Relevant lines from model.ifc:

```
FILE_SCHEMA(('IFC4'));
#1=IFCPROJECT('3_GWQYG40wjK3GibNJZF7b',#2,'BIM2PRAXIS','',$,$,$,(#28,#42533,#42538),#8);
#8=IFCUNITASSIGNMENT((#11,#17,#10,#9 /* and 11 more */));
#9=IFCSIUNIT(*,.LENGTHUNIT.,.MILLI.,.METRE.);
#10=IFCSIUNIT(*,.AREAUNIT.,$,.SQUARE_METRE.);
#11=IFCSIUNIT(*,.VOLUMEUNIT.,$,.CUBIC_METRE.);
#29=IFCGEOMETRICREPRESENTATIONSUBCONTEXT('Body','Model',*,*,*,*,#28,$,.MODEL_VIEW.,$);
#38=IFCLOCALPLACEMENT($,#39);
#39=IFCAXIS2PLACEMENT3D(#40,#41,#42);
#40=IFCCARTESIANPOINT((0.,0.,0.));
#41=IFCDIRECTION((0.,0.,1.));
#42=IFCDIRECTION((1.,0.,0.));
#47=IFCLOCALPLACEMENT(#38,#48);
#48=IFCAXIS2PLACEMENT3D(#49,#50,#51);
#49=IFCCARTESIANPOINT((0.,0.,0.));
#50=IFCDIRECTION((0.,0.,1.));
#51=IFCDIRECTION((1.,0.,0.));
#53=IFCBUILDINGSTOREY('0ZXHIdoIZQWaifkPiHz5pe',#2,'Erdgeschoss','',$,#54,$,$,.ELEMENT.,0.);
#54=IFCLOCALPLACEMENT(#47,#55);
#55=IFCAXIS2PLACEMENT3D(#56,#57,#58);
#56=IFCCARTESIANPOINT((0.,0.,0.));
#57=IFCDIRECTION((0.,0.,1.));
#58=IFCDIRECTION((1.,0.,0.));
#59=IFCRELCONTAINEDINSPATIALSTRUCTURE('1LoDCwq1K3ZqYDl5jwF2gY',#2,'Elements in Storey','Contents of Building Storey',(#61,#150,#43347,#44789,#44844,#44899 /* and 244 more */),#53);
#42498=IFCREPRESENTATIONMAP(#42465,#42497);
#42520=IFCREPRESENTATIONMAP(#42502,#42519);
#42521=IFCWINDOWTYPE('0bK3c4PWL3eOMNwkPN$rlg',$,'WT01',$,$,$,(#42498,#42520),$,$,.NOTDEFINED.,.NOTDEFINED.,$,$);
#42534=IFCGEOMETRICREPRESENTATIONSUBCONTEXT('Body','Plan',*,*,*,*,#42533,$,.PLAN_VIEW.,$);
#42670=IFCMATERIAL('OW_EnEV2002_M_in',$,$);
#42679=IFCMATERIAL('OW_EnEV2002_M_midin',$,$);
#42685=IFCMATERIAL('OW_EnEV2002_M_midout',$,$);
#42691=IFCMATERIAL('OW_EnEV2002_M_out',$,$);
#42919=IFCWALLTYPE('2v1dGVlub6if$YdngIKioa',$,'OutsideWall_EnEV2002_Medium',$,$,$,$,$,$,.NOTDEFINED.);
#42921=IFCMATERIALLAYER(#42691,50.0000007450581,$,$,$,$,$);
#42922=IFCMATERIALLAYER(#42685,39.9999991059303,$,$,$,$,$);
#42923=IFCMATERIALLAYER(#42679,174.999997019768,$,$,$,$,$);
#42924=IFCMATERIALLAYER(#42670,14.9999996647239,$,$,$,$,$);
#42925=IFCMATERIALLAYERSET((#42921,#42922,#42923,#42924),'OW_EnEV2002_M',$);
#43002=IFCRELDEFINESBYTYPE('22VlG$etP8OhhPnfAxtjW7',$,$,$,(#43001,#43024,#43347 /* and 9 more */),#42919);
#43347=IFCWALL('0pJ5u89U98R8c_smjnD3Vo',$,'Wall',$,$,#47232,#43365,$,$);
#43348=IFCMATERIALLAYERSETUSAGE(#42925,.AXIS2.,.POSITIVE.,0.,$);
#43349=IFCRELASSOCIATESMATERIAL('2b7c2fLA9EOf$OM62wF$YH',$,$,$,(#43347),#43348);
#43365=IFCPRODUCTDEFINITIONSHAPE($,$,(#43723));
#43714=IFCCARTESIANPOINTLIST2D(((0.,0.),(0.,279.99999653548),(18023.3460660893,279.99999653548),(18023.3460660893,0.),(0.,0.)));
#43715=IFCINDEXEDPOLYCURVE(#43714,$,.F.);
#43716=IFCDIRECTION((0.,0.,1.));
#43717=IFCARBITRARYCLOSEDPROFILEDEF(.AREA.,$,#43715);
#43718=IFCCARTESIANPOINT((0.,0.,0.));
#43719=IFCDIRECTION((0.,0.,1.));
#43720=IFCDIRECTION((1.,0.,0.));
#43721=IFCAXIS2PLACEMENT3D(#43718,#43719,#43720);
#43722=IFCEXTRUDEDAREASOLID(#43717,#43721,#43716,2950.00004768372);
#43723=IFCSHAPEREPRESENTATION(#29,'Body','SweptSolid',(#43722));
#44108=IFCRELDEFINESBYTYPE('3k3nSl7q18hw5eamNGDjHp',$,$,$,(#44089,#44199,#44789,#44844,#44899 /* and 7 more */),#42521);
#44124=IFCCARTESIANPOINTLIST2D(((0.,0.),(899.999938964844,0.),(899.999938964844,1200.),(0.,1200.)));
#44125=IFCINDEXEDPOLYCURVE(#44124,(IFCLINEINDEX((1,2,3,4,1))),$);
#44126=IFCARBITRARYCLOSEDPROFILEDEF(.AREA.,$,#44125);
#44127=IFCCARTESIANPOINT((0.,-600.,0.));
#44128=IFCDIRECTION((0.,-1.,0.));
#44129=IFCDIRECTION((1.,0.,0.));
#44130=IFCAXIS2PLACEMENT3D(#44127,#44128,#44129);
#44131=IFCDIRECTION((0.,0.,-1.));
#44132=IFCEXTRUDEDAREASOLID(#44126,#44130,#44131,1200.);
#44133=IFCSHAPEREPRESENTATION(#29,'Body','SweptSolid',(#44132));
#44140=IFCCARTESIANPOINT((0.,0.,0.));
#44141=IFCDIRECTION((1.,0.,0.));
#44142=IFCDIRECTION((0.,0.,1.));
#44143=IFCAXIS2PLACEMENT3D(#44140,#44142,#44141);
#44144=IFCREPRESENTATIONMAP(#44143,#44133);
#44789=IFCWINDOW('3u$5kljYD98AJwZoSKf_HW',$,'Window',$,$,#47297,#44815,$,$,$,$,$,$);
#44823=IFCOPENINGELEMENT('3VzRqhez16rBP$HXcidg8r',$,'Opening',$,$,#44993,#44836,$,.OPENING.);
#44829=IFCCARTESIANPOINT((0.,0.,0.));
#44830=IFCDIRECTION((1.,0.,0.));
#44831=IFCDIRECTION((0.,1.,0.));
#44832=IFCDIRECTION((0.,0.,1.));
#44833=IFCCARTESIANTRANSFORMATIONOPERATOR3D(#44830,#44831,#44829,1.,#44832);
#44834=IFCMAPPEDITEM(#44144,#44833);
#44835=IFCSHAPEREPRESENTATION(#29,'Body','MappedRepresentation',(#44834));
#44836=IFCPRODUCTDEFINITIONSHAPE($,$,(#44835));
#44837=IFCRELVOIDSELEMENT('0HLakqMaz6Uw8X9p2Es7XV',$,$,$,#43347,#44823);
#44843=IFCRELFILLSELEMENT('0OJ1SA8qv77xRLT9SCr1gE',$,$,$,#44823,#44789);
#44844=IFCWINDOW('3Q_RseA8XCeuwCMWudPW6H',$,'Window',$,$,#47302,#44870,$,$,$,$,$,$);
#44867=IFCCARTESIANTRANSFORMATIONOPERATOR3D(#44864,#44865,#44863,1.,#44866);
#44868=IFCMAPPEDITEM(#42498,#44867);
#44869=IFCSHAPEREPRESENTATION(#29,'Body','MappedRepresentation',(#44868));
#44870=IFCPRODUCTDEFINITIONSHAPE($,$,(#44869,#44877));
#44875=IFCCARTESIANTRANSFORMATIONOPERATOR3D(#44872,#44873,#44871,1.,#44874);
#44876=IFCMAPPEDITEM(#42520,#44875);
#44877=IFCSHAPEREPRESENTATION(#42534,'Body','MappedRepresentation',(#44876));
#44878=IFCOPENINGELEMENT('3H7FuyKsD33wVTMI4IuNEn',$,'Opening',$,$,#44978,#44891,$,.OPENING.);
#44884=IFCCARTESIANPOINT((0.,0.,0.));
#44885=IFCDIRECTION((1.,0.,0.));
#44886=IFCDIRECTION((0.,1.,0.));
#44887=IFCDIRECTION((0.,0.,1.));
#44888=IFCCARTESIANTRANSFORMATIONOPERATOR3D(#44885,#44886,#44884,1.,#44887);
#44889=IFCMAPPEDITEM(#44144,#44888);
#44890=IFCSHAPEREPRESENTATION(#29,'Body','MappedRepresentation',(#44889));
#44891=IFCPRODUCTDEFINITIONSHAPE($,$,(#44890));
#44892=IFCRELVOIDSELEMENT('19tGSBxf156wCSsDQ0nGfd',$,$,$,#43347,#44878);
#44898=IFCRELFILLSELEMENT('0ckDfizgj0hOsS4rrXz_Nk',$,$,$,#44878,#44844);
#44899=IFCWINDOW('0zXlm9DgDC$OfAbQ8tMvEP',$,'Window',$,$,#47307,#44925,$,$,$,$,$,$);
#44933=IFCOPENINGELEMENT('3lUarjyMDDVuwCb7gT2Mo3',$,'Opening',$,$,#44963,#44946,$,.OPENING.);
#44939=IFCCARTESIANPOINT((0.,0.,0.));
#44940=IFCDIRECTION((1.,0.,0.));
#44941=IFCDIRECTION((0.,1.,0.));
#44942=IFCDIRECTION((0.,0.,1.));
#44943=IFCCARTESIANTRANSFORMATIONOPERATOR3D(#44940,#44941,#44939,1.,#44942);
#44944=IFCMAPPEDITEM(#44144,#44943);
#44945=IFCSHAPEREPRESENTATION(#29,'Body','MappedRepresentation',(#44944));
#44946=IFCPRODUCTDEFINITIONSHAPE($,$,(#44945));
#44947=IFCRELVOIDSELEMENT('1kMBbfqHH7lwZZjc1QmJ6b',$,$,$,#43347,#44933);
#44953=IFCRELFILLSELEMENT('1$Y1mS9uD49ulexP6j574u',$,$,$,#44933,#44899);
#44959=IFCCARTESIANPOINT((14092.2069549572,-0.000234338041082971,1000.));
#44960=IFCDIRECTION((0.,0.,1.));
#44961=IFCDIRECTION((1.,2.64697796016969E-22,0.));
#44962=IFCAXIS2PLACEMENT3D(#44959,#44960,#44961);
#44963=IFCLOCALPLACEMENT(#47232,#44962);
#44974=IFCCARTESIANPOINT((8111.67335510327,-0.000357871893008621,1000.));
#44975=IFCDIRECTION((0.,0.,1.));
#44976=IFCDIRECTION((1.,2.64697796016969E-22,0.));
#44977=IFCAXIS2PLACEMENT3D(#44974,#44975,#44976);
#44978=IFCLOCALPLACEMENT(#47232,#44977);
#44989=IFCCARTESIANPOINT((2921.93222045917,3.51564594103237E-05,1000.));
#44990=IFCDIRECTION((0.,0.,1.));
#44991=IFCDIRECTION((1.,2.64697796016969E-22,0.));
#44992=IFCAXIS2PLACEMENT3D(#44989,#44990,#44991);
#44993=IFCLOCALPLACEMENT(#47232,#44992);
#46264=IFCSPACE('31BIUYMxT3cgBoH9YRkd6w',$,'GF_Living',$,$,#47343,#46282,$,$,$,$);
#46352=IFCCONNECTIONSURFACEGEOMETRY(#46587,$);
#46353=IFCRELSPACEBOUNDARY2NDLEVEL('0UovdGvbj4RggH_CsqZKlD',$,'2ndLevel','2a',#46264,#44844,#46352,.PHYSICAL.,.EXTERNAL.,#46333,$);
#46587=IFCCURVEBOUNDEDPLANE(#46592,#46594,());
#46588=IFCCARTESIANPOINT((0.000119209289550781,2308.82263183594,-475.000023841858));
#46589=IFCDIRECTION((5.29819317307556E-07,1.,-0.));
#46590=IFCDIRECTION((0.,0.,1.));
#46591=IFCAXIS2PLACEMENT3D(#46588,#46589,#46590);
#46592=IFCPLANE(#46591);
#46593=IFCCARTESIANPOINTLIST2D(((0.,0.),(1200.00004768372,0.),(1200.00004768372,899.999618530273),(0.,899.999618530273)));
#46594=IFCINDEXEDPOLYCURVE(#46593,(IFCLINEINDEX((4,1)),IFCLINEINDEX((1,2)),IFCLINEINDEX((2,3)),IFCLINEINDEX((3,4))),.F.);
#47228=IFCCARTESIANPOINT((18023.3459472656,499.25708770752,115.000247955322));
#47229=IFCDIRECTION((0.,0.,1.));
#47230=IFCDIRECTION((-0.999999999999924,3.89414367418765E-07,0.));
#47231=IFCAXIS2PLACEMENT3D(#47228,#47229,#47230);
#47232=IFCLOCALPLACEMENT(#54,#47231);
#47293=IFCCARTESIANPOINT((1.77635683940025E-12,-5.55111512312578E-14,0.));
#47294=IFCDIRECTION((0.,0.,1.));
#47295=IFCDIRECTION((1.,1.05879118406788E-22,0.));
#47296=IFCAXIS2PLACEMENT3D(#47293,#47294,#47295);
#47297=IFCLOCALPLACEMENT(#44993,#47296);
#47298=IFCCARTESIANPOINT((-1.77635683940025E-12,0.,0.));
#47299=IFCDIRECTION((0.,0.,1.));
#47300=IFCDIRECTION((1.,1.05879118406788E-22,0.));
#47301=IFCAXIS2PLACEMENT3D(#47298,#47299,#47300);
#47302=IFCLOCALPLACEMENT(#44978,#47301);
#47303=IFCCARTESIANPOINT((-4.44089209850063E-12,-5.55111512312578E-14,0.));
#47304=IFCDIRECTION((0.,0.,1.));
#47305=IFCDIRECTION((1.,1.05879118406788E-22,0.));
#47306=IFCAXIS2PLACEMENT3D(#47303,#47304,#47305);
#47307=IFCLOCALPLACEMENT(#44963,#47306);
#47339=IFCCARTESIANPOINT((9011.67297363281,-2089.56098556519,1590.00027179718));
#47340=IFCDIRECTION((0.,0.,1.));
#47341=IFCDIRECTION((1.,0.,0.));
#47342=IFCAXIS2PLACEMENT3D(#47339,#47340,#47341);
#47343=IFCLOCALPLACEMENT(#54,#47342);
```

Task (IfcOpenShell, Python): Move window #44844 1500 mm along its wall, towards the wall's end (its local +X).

```python
import numpy as np
import ifcopenshell
import ifcopenshell.api.geometry
import ifcopenshell.util.placement

model = ifcopenshell.open("model.ifc")

window = model.by_guid("3Q_RseA8XCeuwCMWudPW6H")
opening = window.FillsVoids[0].RelatingOpeningElement
wall = opening.VoidsElements[0].RelatingBuildingElement

wall_matrix = ifcopenshell.util.placement.get_local_placement(wall.ObjectPlacement)
shift = wall_matrix[:3, 0] * 1500.0
before = ifcopenshell.util.placement.get_local_placement(window.ObjectPlacement)[:3, 3].copy()

# The window is placed relative to its opening, so it follows when the opening moves.
matrix = ifcopenshell.util.placement.get_local_placement(opening.ObjectPlacement)
matrix[:3, 3] += shift
ifcopenshell.api.geometry.edit_object_placement(
    model, product=opening, matrix=matrix, is_si=False, should_transform_children=True
)

# Space boundary surfaces are stored in each space's coordinates; move them too.
for rel in window.ProvidesBoundaries:
    if not rel.ConnectionGeometry:
        continue
    surface = rel.ConnectionGeometry.SurfaceOnRelatingElement.BasisSurface
    space_matrix = ifcopenshell.util.placement.get_local_placement(rel.RelatingSpace.ObjectPlacement)
    point = np.array(surface.Position.Location.Coordinates) + space_matrix[:3, :3].T @ shift
    surface.Position = model.createIfcAxis2Placement3D(
        model.createIfcCartesianPoint(point.tolist()), surface.Position.Axis, surface.Position.RefDirection
    )

after = ifcopenshell.util.placement.get_local_placement(window.ObjectPlacement)[:3, 3]
print("window moved by", (after - before).round(3) + 0.0)

model.write("model_updated.ifc")
```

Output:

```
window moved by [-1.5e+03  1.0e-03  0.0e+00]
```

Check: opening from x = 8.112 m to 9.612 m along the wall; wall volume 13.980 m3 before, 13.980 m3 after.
